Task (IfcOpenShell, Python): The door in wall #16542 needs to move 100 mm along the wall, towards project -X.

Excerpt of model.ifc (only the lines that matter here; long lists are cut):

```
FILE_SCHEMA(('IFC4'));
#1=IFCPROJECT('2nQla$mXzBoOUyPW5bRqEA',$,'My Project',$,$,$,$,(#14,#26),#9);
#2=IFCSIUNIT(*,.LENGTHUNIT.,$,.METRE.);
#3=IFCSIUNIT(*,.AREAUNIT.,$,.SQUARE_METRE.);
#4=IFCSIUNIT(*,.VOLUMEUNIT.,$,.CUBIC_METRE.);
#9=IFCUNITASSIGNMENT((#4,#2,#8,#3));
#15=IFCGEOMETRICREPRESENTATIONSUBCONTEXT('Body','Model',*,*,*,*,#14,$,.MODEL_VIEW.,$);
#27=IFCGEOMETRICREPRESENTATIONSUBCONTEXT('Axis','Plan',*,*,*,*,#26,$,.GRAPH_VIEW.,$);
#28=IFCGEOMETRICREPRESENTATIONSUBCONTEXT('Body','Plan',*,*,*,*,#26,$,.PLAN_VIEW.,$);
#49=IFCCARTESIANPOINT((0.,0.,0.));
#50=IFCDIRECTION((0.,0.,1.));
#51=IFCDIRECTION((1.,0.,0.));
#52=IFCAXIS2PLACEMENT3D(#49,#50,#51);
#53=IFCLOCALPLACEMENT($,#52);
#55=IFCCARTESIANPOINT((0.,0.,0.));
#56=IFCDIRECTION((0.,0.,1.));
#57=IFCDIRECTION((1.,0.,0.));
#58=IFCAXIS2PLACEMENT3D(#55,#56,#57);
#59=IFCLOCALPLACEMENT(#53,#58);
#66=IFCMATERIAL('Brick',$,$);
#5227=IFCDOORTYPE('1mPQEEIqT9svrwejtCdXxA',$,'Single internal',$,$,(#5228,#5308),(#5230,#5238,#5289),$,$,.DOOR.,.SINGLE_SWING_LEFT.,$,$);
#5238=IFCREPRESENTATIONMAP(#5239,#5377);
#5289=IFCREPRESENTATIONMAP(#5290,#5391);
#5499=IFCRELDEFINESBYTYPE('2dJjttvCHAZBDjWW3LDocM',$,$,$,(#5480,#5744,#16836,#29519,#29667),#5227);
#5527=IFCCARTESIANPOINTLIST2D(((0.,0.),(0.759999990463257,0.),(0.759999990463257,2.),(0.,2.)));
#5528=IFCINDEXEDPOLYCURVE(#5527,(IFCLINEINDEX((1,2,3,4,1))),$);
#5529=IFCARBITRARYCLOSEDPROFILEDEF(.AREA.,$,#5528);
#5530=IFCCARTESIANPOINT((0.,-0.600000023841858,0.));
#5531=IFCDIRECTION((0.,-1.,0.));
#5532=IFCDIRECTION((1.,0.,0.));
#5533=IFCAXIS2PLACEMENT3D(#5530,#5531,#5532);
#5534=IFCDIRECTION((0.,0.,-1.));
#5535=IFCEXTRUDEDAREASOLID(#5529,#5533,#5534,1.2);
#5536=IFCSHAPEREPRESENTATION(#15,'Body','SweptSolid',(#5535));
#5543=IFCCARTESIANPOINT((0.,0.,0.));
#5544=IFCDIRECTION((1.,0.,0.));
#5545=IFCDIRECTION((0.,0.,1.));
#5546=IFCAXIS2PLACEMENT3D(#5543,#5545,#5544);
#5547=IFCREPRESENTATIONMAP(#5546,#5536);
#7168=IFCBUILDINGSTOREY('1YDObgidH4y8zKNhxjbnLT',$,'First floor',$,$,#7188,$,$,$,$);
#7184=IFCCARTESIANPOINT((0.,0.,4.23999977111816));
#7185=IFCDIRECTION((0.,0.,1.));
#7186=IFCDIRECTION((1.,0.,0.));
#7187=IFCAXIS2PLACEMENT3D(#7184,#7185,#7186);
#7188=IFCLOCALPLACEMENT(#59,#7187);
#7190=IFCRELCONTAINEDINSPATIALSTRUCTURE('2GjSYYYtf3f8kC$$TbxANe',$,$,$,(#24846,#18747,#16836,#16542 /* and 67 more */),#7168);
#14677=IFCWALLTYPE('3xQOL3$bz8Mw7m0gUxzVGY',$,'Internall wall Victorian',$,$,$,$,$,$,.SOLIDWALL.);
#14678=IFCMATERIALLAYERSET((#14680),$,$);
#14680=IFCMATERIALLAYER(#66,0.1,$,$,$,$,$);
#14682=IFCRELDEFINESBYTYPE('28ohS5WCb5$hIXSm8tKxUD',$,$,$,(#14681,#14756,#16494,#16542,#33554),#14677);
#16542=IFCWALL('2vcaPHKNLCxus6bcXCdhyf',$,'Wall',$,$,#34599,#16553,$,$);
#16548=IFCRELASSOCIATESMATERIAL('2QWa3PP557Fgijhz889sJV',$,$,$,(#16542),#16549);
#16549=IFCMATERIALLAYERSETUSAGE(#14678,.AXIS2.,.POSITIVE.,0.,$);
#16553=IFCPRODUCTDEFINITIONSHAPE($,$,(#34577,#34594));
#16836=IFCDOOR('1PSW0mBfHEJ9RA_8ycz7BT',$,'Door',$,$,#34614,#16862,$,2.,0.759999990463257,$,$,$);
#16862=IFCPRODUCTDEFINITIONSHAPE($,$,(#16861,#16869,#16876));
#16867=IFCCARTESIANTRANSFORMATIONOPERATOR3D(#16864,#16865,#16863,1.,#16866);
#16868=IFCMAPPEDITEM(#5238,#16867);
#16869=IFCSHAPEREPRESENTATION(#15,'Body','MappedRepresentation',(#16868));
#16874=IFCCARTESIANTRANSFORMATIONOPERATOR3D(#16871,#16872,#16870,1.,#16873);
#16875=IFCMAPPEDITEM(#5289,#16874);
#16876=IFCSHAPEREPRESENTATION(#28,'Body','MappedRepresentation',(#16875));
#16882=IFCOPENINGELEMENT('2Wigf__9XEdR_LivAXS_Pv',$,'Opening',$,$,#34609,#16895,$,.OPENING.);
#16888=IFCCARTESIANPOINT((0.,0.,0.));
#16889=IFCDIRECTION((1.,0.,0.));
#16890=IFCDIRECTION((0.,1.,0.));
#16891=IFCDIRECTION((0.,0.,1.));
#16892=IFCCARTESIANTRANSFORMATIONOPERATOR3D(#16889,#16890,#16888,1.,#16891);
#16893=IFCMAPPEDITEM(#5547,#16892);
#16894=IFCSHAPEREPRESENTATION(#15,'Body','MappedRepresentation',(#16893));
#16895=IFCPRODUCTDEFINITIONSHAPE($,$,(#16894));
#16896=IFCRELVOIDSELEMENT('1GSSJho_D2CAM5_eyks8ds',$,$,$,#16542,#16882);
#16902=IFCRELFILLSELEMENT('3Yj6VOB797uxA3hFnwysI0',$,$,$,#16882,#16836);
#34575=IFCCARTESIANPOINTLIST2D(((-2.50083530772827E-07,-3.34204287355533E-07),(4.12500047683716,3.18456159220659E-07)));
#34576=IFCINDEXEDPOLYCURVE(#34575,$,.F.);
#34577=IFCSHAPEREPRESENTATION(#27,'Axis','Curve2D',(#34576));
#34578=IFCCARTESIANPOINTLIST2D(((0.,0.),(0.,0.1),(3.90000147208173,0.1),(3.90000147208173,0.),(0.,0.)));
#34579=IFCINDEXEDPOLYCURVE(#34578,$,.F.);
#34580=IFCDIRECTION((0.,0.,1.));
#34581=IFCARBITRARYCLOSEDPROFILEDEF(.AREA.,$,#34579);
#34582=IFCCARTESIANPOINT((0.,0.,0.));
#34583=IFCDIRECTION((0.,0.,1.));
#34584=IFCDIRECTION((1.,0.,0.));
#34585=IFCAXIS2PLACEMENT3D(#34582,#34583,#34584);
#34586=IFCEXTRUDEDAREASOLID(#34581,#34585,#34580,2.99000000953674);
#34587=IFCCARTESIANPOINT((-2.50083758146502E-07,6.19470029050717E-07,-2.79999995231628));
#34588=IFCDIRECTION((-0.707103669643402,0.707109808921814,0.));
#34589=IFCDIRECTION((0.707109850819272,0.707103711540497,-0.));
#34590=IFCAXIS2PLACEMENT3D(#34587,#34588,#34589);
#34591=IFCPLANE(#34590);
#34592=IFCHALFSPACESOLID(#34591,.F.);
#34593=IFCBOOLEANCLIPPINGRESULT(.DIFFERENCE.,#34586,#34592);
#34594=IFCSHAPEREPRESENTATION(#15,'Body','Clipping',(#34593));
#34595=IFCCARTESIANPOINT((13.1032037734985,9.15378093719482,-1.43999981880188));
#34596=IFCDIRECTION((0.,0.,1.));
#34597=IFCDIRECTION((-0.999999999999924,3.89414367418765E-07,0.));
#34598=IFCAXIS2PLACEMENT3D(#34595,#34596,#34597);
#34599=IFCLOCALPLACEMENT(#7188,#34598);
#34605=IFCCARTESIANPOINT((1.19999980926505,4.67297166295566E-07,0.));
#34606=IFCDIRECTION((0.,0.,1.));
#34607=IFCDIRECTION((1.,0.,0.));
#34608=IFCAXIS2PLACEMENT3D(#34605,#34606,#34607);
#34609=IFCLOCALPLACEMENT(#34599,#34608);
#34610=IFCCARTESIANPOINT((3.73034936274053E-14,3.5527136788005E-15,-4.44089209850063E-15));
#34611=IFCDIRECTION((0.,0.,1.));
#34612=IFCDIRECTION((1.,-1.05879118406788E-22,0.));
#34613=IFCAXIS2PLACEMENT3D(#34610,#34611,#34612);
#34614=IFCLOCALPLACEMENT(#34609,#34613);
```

```python
import ifcopenshell
import ifcopenshell.api.geometry
import ifcopenshell.util.placement

model = ifcopenshell.open("model.ifc")

door = model.by_id(16836)
opening = door.FillsVoids[0].RelatingOpeningElement
wall = opening.VoidsElements[0].RelatingBuildingElement

wall_matrix = ifcopenshell.util.placement.get_local_placement(wall.ObjectPlacement)
shift = wall_matrix[:3, 0] * 0.1
before = ifcopenshell.util.placement.get_local_placement(door.ObjectPlacement)[:3, 3].copy()

# The door is placed relative to its opening, so it follows when the opening moves.
matrix = ifcopenshell.util.placement.get_local_placement(opening.ObjectPlacement)
matrix[:3, 3] += shift
ifcopenshell.api.geometry.edit_object_placement(
    model, product=opening, matrix=matrix, is_si=False, should_transform_children=True
)

after = ifcopenshell.util.placement.get_local_placement(door.ObjectPlacement)[:3, 3]
print("door moved by", (after - before).round(3) + 0.0)

model.write("model-out.ifc")
```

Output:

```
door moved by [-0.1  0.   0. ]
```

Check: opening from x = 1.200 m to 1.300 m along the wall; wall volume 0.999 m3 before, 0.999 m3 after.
